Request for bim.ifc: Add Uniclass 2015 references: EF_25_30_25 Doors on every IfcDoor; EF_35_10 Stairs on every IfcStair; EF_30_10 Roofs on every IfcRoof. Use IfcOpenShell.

First a look at what the model holds.

```python
import ifcopenshell

model = ifcopenshell.open("bim.ifc")
print(model.schema)
print("classifications:", [c.Name for c in model.by_type("IfcClassification")])
for ifc_class in ("IfcDoor", "IfcRoof", "IfcStair", "IfcWall", "IfcWindow"):
    print(ifc_class, len(model.by_type(ifc_class)))
```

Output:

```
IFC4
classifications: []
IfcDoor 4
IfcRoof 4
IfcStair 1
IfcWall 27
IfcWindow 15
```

```python
import ifcopenshell
import ifcopenshell.api.classification

model = ifcopenshell.open("bim.ifc")

system = ifcopenshell.api.classification.add_classification(model, classification="Uniclass 2015")

codes = {
    "IfcDoor": ("EF_25_30_25", "Doors"),
    "IfcStair": ("EF_35_10", "Stairs"),
    "IfcRoof": ("EF_30_10", "Roofs"),
}
for ifc_class, (code, name) in codes.items():
    products = model.by_type(ifc_class)
    ifcopenshell.api.classification.add_reference(
        model, products=products, classification=system, identification=code, name=name
    )
    print(code, len(products))

model.write("bim_updated.ifc")
```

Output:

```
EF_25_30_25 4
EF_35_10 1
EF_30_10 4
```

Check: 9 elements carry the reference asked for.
